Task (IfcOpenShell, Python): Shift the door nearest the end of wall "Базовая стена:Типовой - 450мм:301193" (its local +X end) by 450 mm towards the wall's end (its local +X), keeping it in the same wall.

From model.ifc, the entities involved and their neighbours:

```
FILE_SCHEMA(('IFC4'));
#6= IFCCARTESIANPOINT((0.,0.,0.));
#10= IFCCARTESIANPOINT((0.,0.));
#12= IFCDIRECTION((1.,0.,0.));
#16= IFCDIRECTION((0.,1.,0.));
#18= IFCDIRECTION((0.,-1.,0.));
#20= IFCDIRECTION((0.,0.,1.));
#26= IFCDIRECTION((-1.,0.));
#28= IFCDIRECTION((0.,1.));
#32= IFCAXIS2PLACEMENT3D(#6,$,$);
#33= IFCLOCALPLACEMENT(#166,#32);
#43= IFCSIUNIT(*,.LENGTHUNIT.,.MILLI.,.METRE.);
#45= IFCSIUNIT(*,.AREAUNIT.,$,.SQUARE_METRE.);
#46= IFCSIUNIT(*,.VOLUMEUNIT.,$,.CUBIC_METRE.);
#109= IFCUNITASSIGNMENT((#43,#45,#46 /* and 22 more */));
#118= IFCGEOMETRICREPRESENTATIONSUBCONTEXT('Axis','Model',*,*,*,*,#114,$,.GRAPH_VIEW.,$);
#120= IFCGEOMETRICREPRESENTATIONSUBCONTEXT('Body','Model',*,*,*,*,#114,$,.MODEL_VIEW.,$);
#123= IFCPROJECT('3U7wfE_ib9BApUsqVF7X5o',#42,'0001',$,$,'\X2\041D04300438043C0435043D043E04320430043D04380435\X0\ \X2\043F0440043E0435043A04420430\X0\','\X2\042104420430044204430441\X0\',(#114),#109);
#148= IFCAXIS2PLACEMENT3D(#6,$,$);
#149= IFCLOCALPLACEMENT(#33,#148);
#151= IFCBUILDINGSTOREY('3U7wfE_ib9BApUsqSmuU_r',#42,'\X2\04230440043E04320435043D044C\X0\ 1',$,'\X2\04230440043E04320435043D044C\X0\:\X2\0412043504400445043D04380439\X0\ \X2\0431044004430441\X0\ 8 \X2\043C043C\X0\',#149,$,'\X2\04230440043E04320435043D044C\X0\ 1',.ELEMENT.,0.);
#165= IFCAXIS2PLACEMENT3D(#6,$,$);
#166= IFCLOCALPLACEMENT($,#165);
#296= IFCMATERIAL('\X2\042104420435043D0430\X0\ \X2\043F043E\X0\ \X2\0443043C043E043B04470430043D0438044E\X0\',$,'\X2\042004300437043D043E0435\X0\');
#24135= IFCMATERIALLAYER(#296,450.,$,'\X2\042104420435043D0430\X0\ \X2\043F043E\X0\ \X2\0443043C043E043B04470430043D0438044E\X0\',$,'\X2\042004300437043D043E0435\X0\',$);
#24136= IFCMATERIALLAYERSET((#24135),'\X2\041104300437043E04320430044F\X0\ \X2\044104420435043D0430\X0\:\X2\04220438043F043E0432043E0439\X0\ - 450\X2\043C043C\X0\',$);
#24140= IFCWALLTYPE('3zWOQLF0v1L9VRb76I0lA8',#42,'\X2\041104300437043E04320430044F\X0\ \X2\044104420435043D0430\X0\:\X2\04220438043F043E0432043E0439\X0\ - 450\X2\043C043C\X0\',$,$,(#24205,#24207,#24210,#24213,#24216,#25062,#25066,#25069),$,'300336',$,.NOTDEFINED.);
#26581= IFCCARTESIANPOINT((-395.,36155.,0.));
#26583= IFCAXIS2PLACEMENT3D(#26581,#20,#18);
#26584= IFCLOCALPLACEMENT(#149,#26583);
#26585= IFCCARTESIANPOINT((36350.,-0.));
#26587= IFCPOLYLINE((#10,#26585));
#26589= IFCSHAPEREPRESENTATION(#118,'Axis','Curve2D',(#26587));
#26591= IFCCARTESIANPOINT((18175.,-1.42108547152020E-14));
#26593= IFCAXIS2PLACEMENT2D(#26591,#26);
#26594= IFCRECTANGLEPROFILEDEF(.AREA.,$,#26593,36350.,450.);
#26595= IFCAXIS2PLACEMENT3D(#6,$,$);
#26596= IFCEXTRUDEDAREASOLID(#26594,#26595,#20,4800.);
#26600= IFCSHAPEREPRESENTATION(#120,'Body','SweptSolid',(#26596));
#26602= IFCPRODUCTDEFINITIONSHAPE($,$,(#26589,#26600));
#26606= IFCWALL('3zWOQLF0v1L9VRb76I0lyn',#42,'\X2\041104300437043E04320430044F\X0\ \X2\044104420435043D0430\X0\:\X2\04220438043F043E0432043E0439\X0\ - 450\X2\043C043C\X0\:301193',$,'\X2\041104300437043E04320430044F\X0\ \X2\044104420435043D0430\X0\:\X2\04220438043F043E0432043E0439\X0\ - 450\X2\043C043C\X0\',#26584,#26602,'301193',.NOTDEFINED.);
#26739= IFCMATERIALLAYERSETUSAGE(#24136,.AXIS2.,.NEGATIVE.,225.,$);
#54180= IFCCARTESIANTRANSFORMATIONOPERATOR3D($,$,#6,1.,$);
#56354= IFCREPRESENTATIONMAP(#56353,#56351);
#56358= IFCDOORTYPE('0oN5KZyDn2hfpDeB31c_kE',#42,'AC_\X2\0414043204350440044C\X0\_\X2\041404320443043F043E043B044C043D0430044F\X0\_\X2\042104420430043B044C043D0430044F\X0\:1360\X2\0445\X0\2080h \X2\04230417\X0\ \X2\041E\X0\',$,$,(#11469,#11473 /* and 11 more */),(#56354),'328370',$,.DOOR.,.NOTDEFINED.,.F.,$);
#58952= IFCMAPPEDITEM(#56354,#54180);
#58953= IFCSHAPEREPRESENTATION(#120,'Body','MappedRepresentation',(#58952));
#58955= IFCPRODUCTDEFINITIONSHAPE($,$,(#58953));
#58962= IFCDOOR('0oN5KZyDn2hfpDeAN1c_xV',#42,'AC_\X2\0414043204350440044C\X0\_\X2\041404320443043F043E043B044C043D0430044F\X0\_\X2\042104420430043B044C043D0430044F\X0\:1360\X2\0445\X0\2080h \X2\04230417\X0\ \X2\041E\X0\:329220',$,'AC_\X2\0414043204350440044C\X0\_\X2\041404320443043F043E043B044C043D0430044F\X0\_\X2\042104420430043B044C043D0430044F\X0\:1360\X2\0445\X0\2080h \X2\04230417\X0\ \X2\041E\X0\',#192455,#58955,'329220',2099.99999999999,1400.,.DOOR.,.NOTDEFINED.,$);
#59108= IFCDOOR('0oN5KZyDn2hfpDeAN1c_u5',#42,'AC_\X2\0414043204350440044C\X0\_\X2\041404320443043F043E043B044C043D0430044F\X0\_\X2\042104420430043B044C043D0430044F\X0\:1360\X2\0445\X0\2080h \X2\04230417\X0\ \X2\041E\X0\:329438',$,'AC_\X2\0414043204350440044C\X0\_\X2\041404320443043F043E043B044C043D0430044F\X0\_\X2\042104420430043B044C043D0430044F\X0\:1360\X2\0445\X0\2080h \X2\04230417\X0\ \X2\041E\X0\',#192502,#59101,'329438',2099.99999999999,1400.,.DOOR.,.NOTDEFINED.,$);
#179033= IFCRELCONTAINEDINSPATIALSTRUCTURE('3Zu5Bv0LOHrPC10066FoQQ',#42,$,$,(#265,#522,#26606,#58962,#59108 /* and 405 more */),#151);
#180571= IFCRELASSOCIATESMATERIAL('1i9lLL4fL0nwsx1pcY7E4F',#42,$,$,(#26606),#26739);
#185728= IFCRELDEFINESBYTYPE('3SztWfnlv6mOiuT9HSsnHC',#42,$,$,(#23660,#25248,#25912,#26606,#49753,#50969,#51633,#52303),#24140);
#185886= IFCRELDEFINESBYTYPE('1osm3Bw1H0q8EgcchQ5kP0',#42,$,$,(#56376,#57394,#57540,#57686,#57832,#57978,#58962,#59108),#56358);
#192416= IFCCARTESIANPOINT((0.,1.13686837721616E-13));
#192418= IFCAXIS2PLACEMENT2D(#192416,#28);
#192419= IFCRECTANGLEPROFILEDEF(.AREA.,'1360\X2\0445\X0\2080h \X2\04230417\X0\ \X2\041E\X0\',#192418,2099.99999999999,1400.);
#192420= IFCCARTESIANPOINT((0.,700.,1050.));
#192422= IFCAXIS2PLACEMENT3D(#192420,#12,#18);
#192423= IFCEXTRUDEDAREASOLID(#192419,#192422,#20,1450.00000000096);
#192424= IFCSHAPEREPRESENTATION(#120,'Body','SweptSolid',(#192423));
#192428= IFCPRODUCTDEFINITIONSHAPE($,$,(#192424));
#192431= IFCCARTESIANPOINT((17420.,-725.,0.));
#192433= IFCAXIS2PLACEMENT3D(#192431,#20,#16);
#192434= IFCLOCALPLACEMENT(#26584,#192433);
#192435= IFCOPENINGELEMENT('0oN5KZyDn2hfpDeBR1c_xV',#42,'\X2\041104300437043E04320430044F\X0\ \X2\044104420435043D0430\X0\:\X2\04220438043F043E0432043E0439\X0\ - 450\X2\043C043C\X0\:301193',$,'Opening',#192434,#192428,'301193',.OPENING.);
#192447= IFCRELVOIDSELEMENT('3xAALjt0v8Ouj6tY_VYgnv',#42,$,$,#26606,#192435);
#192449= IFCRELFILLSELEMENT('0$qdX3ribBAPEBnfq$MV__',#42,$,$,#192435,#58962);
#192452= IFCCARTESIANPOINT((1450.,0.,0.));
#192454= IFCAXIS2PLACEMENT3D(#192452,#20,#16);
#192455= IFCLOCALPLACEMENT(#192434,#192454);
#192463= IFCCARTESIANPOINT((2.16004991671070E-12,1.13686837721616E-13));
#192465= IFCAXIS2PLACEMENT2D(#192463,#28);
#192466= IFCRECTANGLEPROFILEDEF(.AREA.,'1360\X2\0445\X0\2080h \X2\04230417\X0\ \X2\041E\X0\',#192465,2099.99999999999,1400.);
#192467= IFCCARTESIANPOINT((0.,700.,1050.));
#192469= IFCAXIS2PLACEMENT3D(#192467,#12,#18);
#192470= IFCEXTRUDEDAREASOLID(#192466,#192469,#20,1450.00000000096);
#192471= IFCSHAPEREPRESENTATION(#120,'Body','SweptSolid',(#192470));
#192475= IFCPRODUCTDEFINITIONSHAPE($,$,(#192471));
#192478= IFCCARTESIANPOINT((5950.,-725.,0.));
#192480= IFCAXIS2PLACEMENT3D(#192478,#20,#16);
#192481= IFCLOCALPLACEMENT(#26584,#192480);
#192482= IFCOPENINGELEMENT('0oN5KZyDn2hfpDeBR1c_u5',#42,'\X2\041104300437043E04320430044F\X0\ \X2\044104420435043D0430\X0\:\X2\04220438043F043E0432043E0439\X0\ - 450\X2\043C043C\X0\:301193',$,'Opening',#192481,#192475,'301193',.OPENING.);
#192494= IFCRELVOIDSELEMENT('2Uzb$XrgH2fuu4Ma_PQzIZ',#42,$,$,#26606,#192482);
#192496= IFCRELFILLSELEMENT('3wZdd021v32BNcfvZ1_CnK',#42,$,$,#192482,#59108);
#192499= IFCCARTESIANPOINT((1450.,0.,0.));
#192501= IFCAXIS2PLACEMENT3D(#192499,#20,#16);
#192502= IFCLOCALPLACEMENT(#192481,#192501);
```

```python
import ifcopenshell
import ifcopenshell.api.geometry
import ifcopenshell.util.placement
import ifcopenshell.util.unit

model = ifcopenshell.open("model.ifc")
unit_scale = ifcopenshell.util.unit.calculate_unit_scale(model)

door = model.by_guid("0oN5KZyDn2hfpDeAN1c_xV")
opening = door.FillsVoids[0].RelatingOpeningElement
wall = opening.VoidsElements[0].RelatingBuildingElement

wall_matrix = ifcopenshell.util.placement.get_local_placement(wall.ObjectPlacement)
shift = wall_matrix[:3, 0] * 0.45 / unit_scale
before = ifcopenshell.util.placement.get_local_placement(door.ObjectPlacement)[:3, 3].copy()

# The door is placed relative to its opening, so it follows when the opening moves.
matrix = ifcopenshell.util.placement.get_local_placement(opening.ObjectPlacement)
matrix[:3, 3] += shift
ifcopenshell.api.geometry.edit_object_placement(
    model, product=opening, matrix=matrix, is_si=False, should_transform_children=True
)

after = ifcopenshell.util.placement.get_local_placement(door.ObjectPlacement)[:3, 3]
print("door moved by", (after - before).round(3) + 0.0)

model.write("model_updated.ifc")
```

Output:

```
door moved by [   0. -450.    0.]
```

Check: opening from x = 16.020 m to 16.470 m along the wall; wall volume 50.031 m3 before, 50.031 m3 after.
